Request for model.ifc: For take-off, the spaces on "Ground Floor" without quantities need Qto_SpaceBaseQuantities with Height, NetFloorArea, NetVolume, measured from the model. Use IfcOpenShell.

First a look at what the model holds.

```python
import ifcopenshell
import ifcopenshell.util.element
import ifcopenshell.util.unit

model = ifcopenshell.open("model.ifc")
print(model.schema)
for unit_type in ("LENGTHUNIT", "AREAUNIT", "VOLUMEUNIT"):
    print(unit_type, ifcopenshell.util.unit.calculate_unit_scale(model, unit_type))
storey = next(s for s in model.by_type("IfcBuildingStorey") if s.Name == "Ground Floor")
spaces = [e for e in ifcopenshell.util.element.get_decomposition(storey) if e.is_a("IfcSpace")]
for e in sorted(spaces, key=lambda e: e.id()):
    print(e.id(), e.is_a(), e.Name, list(ifcopenshell.util.element.get_psets(e, qtos_only=True)), sep=" | ")
```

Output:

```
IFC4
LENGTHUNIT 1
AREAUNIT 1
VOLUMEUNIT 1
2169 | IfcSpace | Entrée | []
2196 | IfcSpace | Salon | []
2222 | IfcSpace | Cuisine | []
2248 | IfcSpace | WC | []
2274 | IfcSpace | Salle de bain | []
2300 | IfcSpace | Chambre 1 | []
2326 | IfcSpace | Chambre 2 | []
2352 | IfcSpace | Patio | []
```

```python
import ifcopenshell
import ifcopenshell.api.pset
import ifcopenshell.geom
import ifcopenshell.util.element
import ifcopenshell.util.shape
import ifcopenshell.util.unit

model = ifcopenshell.open("model.ifc")
unit_scale = ifcopenshell.util.unit.calculate_unit_scale(model)
area_scale = ifcopenshell.util.unit.calculate_unit_scale(model, "AREAUNIT")
volume_scale = ifcopenshell.util.unit.calculate_unit_scale(model, "VOLUMEUNIT")
settings = ifcopenshell.geom.settings()

storey = next(s for s in model.by_type("IfcBuildingStorey") if s.Name == "Ground Floor")
spaces = [e for e in ifcopenshell.util.element.get_decomposition(storey) if e.is_a("IfcSpace")]

for e in sorted(spaces, key=lambda e: e.id()):
    if ifcopenshell.util.element.get_psets(e, qtos_only=True, should_inherit=False):
        continue
    # Geometry comes back in metres, in the element's own axes.
    shape = ifcopenshell.geom.create_shape(settings, e)
    values = {
        "Height": ifcopenshell.util.shape.get_z(shape.geometry) / unit_scale,
        "NetFloorArea": ifcopenshell.util.shape.get_footprint_area(shape.geometry) / area_scale,
        "NetVolume": ifcopenshell.util.shape.get_volume(shape.geometry) / volume_scale,
    }
    qto = ifcopenshell.api.pset.add_qto(model, product=e, name="Qto_SpaceBaseQuantities")
    ifcopenshell.api.pset.edit_qto(model, qto=qto, properties=values)
    print(e.id(), {k: round(v, 3) for k, v in values.items()})

model.write("model_rev.ifc")
```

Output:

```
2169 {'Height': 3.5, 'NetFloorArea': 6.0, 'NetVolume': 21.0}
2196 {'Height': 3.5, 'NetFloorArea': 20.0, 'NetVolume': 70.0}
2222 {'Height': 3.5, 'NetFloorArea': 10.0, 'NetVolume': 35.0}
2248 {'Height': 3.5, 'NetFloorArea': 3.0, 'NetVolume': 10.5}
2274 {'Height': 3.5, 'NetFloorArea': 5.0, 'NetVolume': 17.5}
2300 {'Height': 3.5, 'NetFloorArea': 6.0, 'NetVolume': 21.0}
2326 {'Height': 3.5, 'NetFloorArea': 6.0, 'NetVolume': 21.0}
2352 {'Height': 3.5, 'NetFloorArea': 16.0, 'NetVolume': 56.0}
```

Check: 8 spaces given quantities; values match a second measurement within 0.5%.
